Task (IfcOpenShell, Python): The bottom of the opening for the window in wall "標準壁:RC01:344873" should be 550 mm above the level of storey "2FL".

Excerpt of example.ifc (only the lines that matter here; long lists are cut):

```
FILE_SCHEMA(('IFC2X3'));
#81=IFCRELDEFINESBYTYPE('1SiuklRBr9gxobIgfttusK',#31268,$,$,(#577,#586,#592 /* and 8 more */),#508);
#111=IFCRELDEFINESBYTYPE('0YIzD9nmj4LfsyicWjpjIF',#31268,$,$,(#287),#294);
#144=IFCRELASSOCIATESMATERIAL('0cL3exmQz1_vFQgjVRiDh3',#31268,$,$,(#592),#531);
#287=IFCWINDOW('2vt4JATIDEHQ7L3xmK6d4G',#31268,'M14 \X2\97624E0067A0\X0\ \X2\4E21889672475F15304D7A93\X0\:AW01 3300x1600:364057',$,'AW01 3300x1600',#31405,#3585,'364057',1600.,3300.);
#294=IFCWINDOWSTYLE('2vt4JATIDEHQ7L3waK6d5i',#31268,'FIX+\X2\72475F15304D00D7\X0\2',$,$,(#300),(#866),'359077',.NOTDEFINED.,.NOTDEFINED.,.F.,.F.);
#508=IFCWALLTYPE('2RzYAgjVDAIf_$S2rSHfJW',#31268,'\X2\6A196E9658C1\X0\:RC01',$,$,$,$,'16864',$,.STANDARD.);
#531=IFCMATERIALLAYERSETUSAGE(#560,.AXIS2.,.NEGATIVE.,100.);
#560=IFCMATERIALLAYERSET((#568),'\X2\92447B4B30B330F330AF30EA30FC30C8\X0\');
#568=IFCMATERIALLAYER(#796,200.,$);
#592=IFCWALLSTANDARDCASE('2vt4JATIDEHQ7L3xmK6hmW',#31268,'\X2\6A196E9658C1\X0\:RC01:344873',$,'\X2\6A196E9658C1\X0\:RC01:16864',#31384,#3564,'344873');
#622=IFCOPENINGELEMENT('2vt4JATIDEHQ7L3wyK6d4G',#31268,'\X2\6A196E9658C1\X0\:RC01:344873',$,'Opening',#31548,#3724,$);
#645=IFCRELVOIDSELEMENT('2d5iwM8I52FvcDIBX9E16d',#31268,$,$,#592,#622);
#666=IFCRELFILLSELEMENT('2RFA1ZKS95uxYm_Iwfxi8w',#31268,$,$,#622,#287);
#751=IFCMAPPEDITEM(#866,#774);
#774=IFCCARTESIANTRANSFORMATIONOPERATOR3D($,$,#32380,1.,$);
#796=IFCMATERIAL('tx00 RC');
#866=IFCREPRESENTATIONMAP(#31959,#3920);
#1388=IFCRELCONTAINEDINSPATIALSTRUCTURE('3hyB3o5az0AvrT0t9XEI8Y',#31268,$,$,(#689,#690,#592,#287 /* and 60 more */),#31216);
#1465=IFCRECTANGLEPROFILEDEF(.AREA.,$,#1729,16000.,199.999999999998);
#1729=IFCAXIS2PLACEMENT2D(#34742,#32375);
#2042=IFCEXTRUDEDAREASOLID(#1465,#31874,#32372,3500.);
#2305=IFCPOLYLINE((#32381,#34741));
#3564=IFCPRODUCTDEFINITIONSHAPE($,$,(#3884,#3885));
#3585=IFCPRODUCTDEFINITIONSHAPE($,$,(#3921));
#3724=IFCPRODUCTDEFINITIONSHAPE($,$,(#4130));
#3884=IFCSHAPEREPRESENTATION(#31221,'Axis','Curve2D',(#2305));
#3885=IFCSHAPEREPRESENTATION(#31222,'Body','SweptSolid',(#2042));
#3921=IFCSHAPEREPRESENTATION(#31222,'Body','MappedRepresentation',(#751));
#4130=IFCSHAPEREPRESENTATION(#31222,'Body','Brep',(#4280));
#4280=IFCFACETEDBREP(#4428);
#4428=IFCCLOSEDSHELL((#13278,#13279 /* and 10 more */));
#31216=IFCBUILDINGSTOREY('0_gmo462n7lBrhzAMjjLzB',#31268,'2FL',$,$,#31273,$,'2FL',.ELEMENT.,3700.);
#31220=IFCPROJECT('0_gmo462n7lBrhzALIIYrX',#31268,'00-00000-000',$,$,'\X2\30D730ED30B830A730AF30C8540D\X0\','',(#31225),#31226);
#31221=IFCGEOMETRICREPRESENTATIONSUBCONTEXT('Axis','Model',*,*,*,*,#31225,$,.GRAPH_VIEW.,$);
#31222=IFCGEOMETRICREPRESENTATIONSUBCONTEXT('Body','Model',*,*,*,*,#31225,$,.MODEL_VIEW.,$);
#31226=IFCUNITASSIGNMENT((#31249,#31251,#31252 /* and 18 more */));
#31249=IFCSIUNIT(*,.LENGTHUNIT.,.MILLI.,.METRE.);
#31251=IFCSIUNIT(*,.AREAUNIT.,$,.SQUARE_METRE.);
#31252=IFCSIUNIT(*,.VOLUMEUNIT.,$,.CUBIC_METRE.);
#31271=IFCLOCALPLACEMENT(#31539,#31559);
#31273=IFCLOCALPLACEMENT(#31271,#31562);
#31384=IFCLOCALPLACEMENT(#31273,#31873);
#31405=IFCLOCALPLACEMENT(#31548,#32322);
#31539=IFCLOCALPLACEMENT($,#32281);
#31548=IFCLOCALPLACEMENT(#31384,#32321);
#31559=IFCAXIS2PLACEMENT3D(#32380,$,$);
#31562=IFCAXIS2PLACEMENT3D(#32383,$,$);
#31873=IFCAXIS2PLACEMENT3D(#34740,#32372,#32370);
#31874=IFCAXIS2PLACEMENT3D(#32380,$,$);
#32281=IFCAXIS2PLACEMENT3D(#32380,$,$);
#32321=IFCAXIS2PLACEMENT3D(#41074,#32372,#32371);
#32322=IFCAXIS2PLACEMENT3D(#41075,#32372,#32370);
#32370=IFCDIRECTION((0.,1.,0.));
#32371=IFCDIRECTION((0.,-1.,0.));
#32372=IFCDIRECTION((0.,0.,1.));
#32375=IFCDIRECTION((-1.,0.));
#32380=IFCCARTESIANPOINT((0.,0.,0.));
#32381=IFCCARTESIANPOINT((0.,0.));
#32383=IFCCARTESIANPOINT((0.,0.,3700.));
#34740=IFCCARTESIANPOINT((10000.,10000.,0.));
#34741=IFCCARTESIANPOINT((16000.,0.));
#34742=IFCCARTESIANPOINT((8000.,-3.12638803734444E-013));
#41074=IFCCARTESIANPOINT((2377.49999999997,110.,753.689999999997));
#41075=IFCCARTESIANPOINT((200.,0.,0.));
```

```python
import numpy as np
import ifcopenshell
import ifcopenshell.api.geometry
import ifcopenshell.geom
import ifcopenshell.util.element
import ifcopenshell.util.placement
import ifcopenshell.util.shape
import ifcopenshell.util.unit

model = ifcopenshell.open("example.ifc")
unit_scale = ifcopenshell.util.unit.calculate_unit_scale(model)

window = model.by_id(287)
opening = window.FillsVoids[0].RelatingOpeningElement
storey = ifcopenshell.util.element.get_container(window, ifc_class="IfcBuildingStorey")
level = ifcopenshell.util.placement.get_local_placement(storey.ObjectPlacement)[2, 3]

# The opening's origin need not be at the sill, so measure its lowest point.
shape = ifcopenshell.geom.create_shape(ifcopenshell.geom.settings(), opening)
bottom = ifcopenshell.util.shape.get_shape_bottom_elevation(shape, shape.geometry) / unit_scale
dz = level + 0.55 / unit_scale - bottom

shift = np.array([0.0, 0.0, dz])
# The window is placed relative to its opening, so it follows when the opening moves.
matrix = ifcopenshell.util.placement.get_local_placement(opening.ObjectPlacement)
matrix[:3, 3] += shift
ifcopenshell.api.geometry.edit_object_placement(
    model, product=opening, matrix=matrix, is_si=False, should_transform_children=True
)

print(f"moved by {dz * unit_scale:+.3f} m")

model.write("example_rev.ifc")
```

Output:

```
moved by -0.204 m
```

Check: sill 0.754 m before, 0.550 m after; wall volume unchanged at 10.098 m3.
